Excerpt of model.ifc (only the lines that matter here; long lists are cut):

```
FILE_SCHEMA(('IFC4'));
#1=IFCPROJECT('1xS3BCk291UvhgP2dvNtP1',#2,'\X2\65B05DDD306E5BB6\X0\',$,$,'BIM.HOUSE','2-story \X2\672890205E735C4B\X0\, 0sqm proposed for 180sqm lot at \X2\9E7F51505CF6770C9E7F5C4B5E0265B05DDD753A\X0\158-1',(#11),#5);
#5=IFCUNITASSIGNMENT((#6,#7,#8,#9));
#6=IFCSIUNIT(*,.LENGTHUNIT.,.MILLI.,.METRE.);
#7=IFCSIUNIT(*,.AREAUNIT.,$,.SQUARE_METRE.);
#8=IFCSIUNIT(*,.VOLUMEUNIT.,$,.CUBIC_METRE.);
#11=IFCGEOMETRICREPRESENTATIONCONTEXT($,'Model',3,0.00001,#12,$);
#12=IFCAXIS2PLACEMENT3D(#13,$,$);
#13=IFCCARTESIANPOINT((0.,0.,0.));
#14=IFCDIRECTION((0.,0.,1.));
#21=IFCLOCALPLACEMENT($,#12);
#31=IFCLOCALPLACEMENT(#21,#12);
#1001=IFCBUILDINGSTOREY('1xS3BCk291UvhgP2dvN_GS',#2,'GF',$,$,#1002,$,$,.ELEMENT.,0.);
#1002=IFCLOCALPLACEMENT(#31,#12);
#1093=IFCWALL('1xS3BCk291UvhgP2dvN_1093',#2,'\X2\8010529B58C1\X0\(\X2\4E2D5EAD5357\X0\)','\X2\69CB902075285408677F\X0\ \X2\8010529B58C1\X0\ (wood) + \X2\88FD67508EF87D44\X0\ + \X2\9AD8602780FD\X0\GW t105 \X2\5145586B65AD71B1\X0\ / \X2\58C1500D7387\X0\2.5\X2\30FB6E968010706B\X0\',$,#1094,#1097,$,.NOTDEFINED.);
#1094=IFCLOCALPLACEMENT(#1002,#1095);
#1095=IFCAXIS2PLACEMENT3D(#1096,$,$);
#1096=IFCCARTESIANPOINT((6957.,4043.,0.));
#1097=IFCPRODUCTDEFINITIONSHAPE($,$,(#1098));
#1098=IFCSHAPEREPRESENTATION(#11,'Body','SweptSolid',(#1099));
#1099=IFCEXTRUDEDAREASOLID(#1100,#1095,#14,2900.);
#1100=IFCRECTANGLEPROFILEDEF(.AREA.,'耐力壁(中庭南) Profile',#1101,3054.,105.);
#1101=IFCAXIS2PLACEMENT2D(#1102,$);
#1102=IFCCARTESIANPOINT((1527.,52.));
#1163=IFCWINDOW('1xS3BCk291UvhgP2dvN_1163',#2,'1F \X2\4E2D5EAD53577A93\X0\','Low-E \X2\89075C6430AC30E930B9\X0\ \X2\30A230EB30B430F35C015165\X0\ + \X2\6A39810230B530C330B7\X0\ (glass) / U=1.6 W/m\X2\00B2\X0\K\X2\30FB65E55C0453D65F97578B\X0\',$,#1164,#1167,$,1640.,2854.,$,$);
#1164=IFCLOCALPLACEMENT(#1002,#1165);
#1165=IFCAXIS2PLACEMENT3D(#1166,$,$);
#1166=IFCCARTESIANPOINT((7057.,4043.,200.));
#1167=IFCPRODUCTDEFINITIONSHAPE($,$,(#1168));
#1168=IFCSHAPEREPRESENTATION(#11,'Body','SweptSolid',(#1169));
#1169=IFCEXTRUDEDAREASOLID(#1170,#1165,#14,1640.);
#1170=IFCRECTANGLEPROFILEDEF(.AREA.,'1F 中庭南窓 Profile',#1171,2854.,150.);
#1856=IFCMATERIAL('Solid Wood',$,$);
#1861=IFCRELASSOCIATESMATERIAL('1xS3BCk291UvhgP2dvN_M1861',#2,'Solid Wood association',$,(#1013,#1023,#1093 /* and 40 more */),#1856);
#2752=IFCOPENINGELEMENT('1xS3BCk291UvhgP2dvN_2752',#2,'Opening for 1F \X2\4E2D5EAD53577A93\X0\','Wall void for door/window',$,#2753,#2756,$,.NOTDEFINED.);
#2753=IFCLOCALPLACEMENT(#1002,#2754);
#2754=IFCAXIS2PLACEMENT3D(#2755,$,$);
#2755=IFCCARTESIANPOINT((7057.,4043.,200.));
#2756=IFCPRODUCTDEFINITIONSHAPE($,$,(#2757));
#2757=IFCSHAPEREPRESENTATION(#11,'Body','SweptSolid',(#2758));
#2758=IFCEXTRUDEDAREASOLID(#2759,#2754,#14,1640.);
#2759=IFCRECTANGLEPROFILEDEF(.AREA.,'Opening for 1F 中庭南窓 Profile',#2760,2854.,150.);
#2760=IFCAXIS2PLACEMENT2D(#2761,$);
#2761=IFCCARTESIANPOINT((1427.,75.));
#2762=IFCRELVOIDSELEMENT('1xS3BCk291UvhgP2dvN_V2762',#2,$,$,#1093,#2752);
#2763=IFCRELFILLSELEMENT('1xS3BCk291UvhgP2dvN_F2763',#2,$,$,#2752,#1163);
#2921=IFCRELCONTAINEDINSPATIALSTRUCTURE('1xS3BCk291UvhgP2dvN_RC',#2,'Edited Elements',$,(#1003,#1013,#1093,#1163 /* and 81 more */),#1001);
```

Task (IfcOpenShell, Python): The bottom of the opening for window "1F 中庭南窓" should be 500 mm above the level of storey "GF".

```python
import numpy as np
import ifcopenshell
import ifcopenshell.api.geometry
import ifcopenshell.geom
import ifcopenshell.util.element
import ifcopenshell.util.placement
import ifcopenshell.util.shape
import ifcopenshell.util.unit

model = ifcopenshell.open("model.ifc")
unit_scale = ifcopenshell.util.unit.calculate_unit_scale(model)

window = model.by_guid("1xS3BCk291UvhgP2dvN_1163")
opening = window.FillsVoids[0].RelatingOpeningElement
storey = ifcopenshell.util.element.get_container(window, ifc_class="IfcBuildingStorey")
level = ifcopenshell.util.placement.get_local_placement(storey.ObjectPlacement)[2, 3]

# The opening's origin need not be at the sill, so measure its lowest point.
shape = ifcopenshell.geom.create_shape(ifcopenshell.geom.settings(), opening)
bottom = ifcopenshell.util.shape.get_shape_bottom_elevation(shape, shape.geometry) / unit_scale
dz = level + 0.5 / unit_scale - bottom

shift = np.array([0.0, 0.0, dz])
# The window is not placed relative to its opening, so move both.
for product in (opening, window):
    matrix = ifcopenshell.util.placement.get_local_placement(product.ObjectPlacement)
    matrix[:3, 3] += shift
    ifcopenshell.api.geometry.edit_object_placement(model, product=product, matrix=matrix, is_si=False)

print(f"moved by {dz * unit_scale:+.3f} m")

model.write("model_edited.ifc")
```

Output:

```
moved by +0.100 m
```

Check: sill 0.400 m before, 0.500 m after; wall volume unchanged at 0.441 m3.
